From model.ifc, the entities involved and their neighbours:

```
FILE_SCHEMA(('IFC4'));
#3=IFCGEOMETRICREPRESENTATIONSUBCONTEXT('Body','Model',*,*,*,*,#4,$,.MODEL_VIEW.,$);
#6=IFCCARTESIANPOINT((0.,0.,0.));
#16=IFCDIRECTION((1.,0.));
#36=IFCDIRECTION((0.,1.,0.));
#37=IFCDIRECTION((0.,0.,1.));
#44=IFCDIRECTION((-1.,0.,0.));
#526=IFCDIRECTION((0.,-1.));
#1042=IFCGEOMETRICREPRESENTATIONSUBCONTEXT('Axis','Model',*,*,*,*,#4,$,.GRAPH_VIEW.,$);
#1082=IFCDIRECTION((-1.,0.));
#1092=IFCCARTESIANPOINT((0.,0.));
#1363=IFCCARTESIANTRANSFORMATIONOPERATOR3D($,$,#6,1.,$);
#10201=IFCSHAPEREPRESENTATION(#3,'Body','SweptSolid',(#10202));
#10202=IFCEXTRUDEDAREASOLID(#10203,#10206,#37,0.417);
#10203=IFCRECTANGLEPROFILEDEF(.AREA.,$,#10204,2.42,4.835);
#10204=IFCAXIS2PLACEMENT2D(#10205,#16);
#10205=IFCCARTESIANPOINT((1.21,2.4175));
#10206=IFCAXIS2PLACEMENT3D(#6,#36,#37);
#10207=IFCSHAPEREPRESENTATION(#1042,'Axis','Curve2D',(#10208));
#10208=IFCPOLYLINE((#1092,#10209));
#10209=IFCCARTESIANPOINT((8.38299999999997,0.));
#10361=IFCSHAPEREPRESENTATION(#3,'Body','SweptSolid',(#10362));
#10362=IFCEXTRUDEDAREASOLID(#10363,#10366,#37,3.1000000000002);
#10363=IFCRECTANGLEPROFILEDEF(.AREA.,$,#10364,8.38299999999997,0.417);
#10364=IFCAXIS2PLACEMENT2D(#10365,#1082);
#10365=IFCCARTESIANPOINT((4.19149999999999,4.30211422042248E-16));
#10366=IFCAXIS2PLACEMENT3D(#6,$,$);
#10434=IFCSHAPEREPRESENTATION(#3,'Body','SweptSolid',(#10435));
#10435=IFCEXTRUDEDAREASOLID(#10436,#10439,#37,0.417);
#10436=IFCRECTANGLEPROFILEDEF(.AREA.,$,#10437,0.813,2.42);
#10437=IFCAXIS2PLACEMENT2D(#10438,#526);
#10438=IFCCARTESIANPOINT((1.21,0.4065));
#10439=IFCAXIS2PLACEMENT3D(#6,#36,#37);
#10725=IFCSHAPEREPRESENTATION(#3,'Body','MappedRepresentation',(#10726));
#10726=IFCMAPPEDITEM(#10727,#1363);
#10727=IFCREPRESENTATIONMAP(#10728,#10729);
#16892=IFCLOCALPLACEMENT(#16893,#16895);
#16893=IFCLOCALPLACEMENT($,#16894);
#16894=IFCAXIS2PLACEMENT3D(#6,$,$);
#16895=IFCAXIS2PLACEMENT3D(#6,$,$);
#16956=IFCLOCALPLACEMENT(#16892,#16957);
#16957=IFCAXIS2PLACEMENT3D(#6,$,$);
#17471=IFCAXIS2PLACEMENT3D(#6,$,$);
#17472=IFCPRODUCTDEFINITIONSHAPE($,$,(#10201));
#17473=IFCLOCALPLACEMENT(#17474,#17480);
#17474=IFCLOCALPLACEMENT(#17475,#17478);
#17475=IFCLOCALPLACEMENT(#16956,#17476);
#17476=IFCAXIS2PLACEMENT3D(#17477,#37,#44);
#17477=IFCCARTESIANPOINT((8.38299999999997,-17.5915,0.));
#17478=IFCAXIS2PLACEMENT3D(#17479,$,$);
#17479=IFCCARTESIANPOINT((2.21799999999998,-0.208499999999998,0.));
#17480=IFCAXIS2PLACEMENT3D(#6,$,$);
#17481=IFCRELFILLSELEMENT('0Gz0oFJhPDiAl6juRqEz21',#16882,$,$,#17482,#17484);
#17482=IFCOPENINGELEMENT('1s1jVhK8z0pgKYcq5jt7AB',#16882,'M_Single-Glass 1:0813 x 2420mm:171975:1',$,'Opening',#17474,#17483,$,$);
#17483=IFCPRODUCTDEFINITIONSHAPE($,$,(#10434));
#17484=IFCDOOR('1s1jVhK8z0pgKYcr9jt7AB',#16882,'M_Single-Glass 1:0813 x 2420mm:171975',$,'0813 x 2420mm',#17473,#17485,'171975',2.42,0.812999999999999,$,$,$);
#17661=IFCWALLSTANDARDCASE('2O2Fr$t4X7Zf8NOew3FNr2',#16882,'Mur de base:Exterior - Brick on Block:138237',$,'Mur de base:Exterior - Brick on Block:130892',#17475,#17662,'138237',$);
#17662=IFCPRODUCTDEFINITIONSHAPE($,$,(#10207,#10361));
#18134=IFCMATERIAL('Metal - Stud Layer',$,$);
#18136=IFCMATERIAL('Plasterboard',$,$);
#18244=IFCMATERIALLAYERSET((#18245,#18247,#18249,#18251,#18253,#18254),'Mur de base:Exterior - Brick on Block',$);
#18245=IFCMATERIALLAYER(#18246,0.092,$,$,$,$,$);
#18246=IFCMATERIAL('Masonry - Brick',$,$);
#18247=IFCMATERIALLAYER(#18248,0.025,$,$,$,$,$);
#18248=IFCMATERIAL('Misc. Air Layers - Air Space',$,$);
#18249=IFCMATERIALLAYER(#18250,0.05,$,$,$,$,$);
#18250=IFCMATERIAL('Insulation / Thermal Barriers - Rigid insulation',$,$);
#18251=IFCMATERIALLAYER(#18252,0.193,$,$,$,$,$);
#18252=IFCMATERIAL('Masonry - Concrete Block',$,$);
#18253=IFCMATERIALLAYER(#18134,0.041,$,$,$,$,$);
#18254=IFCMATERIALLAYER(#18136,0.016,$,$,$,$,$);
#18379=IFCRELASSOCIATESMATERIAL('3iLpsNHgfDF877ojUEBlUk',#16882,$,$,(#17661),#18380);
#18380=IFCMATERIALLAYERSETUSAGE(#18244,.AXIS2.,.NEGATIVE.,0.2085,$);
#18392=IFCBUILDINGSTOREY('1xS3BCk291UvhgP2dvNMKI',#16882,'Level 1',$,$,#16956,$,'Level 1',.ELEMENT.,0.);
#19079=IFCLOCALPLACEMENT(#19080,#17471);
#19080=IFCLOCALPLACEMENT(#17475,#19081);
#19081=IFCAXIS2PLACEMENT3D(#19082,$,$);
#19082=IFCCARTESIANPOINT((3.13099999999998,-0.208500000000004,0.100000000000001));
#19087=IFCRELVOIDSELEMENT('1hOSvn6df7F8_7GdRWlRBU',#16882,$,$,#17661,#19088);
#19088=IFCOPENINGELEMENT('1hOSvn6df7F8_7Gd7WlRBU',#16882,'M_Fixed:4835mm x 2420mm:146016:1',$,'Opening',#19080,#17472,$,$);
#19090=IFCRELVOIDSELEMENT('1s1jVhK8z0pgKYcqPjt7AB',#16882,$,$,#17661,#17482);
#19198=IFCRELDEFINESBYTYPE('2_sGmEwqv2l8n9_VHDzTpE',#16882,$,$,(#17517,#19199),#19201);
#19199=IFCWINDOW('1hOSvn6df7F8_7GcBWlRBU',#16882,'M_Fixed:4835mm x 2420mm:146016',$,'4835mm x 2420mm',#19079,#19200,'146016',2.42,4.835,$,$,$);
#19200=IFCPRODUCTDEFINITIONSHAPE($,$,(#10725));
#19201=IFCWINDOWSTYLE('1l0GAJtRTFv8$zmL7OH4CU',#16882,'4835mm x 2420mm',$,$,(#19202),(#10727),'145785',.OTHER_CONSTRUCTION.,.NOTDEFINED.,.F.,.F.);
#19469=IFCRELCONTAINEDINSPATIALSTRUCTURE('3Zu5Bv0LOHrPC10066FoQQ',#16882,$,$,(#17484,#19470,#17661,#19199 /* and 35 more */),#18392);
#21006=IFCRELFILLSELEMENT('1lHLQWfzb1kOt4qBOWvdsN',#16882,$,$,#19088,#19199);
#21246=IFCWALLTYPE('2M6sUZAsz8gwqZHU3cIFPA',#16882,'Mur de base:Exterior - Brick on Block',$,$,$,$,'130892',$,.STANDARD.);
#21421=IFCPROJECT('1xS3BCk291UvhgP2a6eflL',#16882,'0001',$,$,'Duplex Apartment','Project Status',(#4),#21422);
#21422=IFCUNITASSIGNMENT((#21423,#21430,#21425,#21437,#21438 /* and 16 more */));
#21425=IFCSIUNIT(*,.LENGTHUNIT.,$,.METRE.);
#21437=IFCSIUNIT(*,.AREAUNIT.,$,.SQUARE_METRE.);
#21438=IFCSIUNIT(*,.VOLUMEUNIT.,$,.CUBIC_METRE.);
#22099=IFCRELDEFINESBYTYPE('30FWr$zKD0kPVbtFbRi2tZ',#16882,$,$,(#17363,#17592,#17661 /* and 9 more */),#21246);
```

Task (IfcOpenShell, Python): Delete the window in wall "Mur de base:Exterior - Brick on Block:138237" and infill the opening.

```python
import ifcopenshell
import ifcopenshell.api.feature
import ifcopenshell.api.root
import ifcopenshell.geom
import ifcopenshell.util.shape

model = ifcopenshell.open("model.ifc")
settings = ifcopenshell.geom.settings()


def volume(element):
    """Net volume in cubic metres, openings subtracted."""
    shape = ifcopenshell.geom.create_shape(settings, element)
    return ifcopenshell.util.shape.get_volume(shape.geometry)


window = model.by_guid("1hOSvn6df7F8_7GcBWlRBU")
opening = window.FillsVoids[0].RelatingOpeningElement
wall = opening.VoidsElements[0].RelatingBuildingElement
before = volume(wall)

ifcopenshell.api.root.remove_product(model, product=window)
ifcopenshell.api.feature.remove_feature(model, feature=opening)

after = volume(wall)

print(f"wall volume {before:.3f} -> {after:.3f} m3")

model.write("model_edited.ifc")
```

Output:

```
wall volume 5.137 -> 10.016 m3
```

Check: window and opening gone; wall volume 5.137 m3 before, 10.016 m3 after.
